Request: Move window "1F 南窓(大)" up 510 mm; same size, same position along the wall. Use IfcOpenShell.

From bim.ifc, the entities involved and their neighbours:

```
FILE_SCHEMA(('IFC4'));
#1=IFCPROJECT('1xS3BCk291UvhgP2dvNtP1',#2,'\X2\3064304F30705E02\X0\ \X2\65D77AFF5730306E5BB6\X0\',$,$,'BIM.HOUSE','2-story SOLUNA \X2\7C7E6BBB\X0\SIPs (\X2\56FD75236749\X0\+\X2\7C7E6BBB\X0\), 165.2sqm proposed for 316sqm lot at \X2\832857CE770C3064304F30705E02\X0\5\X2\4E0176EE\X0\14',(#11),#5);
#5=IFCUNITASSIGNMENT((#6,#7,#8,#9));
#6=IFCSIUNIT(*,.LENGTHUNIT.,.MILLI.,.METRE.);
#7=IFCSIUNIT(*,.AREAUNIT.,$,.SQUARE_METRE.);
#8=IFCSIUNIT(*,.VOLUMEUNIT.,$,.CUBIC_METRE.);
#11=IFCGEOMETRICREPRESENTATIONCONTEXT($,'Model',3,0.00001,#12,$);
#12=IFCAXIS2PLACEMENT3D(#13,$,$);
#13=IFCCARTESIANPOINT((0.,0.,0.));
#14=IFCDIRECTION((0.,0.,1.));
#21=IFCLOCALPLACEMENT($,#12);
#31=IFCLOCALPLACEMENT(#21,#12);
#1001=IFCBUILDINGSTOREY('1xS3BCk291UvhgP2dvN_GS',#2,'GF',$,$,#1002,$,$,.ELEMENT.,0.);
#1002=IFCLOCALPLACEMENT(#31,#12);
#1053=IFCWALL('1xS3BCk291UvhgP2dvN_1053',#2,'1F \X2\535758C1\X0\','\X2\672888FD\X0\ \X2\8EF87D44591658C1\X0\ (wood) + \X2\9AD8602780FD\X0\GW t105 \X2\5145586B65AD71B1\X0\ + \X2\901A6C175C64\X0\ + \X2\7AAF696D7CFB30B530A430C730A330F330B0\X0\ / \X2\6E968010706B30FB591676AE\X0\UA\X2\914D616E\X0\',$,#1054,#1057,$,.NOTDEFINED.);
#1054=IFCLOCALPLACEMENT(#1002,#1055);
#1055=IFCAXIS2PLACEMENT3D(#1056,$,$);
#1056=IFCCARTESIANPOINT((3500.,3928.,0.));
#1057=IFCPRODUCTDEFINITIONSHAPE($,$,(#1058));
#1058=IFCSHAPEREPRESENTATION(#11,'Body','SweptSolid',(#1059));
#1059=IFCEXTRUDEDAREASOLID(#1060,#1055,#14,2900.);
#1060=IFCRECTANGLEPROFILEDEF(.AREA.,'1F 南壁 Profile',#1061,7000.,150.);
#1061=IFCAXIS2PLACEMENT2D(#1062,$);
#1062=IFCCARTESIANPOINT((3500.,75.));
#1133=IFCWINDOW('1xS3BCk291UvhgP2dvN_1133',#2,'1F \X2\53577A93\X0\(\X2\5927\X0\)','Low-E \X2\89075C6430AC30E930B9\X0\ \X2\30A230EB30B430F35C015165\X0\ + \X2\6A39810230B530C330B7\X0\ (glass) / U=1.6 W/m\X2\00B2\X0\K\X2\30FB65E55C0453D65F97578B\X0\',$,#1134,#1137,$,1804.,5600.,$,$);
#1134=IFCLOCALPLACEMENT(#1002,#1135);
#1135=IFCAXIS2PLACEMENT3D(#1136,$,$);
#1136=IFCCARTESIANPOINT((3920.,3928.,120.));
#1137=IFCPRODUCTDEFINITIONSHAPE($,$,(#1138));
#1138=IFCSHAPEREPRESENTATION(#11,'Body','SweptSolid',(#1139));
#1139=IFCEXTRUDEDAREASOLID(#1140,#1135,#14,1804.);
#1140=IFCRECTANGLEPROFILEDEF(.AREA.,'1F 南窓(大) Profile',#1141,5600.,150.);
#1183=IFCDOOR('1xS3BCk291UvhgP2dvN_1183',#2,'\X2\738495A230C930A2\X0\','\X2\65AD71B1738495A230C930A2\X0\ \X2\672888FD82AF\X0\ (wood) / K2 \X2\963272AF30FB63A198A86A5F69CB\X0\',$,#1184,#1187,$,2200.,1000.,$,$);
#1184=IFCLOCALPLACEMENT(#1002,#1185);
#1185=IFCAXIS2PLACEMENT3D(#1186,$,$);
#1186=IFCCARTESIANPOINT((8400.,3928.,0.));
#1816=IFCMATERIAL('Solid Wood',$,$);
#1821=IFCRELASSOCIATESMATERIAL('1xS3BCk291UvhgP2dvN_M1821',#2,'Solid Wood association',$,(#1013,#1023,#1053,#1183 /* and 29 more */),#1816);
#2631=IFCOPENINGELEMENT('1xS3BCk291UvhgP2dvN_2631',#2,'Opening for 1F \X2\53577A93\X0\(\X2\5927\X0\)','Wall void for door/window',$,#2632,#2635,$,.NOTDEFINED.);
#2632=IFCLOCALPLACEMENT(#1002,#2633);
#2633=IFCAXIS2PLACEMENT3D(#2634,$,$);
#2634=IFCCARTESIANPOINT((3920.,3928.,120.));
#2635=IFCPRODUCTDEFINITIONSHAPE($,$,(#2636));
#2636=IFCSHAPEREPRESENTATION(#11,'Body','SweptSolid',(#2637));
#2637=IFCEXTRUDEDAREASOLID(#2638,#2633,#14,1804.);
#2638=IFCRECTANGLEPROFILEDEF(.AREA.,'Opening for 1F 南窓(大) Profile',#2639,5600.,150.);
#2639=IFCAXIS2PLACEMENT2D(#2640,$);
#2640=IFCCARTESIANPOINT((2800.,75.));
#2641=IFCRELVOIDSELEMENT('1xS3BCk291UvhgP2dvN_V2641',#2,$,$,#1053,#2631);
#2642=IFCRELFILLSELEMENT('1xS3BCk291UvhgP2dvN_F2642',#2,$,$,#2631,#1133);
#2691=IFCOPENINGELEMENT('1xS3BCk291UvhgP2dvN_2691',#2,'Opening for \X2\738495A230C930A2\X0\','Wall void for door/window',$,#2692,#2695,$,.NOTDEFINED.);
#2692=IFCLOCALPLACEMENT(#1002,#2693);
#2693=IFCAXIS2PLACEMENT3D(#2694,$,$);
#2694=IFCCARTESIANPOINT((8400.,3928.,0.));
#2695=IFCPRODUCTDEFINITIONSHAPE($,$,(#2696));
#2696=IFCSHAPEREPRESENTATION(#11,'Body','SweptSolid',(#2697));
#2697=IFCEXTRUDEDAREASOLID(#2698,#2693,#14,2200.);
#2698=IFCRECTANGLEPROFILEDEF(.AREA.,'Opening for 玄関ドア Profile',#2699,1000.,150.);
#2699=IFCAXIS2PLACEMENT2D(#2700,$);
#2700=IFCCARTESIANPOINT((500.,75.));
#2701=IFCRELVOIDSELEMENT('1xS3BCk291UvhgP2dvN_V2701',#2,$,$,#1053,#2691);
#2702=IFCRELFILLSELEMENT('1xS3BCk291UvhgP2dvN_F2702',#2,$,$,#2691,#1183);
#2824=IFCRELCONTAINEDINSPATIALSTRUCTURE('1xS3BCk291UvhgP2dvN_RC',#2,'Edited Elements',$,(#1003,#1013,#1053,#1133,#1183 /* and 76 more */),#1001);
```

```python
import numpy as np
import ifcopenshell
import ifcopenshell.api.geometry
import ifcopenshell.util.placement
import ifcopenshell.util.unit

model = ifcopenshell.open("bim.ifc")
unit_scale = ifcopenshell.util.unit.calculate_unit_scale(model)

window = model.by_guid("1xS3BCk291UvhgP2dvN_1133")
opening = window.FillsVoids[0].RelatingOpeningElement
dz = 510.0

shift = np.array([0.0, 0.0, dz])
# The window is not placed relative to its opening, so move both.
for product in (opening, window):
    matrix = ifcopenshell.util.placement.get_local_placement(product.ObjectPlacement)
    matrix[:3, 3] += shift
    ifcopenshell.api.geometry.edit_object_placement(model, product=product, matrix=matrix, is_si=False)

print(f"moved by {dz * unit_scale:+.3f} m")

model.write("bim_updated.ifc")
```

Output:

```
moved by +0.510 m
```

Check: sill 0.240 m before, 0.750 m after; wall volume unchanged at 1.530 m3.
